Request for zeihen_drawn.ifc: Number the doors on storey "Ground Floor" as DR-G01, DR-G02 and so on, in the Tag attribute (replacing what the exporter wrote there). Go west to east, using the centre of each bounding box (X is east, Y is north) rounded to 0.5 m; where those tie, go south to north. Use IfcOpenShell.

First a look at what the model holds.

```python
import ifcopenshell
import ifcopenshell.util.element
import ifcopenshell.util.placement

model = ifcopenshell.open("zeihen_drawn.ifc")
print(model.schema)
storey = next(s for s in model.by_type("IfcBuildingStorey") if s.Name == "Ground Floor")
doors = [e for e in ifcopenshell.util.element.get_decomposition(storey) if e.is_a("IfcDoor")]
for e in sorted(doors, key=lambda e: e.id()):
    origin = ifcopenshell.util.placement.get_local_placement(e.ObjectPlacement)[:3, 3]
    print(e.id(), e.Tag, e.Name, origin.round(2) + 0.0, sep=" | ")
```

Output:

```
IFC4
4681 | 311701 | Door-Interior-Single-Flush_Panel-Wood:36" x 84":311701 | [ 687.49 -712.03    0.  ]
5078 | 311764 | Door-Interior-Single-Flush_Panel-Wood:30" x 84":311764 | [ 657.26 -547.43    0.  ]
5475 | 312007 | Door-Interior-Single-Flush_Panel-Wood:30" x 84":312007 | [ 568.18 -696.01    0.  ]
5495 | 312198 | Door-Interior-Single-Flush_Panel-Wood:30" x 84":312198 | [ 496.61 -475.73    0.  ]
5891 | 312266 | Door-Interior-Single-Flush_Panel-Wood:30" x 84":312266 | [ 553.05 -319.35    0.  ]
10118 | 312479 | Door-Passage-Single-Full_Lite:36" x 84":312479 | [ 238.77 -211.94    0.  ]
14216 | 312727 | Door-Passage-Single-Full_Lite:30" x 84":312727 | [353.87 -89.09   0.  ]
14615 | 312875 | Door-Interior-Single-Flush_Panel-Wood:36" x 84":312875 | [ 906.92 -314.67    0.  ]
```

```python
import ifcopenshell
import ifcopenshell.geom
import ifcopenshell.util.element
import ifcopenshell.util.shape

model = ifcopenshell.open("zeihen_drawn.ifc")
settings = ifcopenshell.geom.settings()
settings.set("use-world-coords", True)


def centre(element):
    shape = ifcopenshell.geom.create_shape(settings, element)
    return ifcopenshell.util.shape.get_bbox_centroid(shape.geometry)


storey = next(s for s in model.by_type("IfcBuildingStorey") if s.Name == "Ground Floor")
doors = [e for e in ifcopenshell.util.element.get_decomposition(storey) if e.is_a("IfcDoor")]

# Insertion points can sit at a corner or the storey origin, so sort by the geometry (in metres).
centres = {e: centre(e) for e in doors}
doors.sort(key=lambda e: (round(centres[e][0] / 0.5), centres[e][1]))

for i, e in enumerate(doors, start=1):
    number = f"DR-G{i:02d}"
    e.Tag = number
    print(e.id(), number)

model.write("zeihen_drawn_updated.ifc")
```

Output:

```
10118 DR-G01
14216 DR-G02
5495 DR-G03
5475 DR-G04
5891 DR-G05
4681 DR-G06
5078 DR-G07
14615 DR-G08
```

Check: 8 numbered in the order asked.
